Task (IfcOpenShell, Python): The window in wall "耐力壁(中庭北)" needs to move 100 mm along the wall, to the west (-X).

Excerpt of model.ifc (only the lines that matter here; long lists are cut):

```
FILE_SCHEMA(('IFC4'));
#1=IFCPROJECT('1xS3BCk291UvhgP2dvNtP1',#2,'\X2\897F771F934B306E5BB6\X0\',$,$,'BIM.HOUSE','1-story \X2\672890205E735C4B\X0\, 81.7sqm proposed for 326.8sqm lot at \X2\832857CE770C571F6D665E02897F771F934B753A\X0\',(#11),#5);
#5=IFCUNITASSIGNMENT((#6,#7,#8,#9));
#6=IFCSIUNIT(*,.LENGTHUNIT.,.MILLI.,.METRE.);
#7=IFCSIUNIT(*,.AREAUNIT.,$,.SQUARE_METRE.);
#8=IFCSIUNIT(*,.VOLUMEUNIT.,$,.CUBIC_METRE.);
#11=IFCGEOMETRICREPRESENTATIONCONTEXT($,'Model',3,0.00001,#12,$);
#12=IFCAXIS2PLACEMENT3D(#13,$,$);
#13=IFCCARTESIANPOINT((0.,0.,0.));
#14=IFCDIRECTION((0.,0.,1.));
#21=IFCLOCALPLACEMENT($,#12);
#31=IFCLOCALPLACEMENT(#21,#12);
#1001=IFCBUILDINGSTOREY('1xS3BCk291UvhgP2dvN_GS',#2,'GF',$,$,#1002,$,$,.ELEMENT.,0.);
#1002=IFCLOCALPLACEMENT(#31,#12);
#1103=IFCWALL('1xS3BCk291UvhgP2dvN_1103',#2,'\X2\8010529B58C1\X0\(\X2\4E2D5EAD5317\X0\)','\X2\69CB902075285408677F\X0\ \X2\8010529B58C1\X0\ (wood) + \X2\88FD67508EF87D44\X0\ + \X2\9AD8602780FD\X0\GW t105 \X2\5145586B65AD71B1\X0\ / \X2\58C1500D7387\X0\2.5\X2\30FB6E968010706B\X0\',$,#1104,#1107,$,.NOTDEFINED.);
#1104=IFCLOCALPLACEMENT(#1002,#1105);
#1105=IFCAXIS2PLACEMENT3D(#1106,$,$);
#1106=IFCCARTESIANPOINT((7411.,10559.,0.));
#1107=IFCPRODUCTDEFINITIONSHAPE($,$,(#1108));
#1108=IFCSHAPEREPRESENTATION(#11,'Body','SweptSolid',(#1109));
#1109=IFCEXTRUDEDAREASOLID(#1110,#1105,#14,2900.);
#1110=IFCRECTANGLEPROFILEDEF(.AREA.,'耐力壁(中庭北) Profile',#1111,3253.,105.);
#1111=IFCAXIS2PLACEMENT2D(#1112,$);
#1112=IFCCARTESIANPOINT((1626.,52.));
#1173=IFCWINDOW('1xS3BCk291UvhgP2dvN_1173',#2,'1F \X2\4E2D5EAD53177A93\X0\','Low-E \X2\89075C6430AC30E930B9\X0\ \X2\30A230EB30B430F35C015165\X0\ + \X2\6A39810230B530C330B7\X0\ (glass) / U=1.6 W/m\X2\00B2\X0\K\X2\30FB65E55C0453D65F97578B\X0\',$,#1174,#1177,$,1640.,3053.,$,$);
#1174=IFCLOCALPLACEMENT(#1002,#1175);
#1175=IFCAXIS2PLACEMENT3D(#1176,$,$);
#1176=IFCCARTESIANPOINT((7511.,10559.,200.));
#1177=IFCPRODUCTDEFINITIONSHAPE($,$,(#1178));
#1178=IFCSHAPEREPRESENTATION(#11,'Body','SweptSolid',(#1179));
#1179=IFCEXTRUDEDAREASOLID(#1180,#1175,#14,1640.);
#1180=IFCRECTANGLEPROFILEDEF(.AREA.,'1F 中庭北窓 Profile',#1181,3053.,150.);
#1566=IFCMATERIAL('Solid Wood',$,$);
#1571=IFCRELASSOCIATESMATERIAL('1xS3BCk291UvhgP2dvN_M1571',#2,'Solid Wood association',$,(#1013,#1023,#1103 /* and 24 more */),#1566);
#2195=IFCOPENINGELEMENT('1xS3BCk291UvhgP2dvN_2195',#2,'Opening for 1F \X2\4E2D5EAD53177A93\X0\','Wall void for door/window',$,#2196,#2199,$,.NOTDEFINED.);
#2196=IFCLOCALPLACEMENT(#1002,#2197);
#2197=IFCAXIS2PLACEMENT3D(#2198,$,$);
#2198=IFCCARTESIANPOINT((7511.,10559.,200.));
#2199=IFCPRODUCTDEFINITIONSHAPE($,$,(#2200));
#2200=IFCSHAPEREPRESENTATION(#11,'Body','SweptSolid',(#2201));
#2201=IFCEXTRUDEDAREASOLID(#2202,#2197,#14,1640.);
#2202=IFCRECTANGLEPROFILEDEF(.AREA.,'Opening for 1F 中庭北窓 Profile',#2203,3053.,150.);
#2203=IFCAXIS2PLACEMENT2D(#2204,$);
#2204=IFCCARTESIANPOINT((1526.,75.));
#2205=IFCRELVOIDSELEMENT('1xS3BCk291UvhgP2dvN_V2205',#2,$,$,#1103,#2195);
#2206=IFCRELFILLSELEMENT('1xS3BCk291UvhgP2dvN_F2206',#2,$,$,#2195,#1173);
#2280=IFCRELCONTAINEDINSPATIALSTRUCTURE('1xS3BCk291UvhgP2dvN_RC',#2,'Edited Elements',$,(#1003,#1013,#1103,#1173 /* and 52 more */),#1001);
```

```python
import ifcopenshell
import ifcopenshell.api.geometry
import ifcopenshell.util.placement

model = ifcopenshell.open("model.ifc")

window = model.by_guid("1xS3BCk291UvhgP2dvN_1173")
opening = window.FillsVoids[0].RelatingOpeningElement
wall = opening.VoidsElements[0].RelatingBuildingElement

wall_matrix = ifcopenshell.util.placement.get_local_placement(wall.ObjectPlacement)
shift = wall_matrix[:3, 0] * -100.0
before = ifcopenshell.util.placement.get_local_placement(window.ObjectPlacement)[:3, 3].copy()

# The window is not placed relative to its opening, so move both.
for product in (opening, window):
    matrix = ifcopenshell.util.placement.get_local_placement(product.ObjectPlacement)
    matrix[:3, 3] += shift
    ifcopenshell.api.geometry.edit_object_placement(model, product=product, matrix=matrix, is_si=False)

after = ifcopenshell.util.placement.get_local_placement(window.ObjectPlacement)[:3, 3]
print("window moved by", (after - before).round(3) + 0.0)

model.write("model-out.ifc")
```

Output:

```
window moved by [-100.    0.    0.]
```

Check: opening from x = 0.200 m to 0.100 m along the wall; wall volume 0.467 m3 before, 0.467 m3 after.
